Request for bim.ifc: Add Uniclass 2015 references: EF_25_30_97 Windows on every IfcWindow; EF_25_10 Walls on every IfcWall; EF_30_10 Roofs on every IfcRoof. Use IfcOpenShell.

First a look at what the model holds.

```python
import ifcopenshell

model = ifcopenshell.open("bim.ifc")
print(model.schema)
print("classifications:", [c.Name for c in model.by_type("IfcClassification")])
for ifc_class in ("IfcDoor", "IfcRoof", "IfcStair", "IfcWall", "IfcWindow"):
    print(ifc_class, len(model.by_type(ifc_class)))
```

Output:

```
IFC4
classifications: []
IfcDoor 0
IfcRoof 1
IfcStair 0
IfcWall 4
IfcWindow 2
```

```python
import ifcopenshell
import ifcopenshell.api.classification

model = ifcopenshell.open("bim.ifc")

system = ifcopenshell.api.classification.add_classification(model, classification="Uniclass 2015")

codes = {
    "IfcWindow": ("EF_25_30_97", "Windows"),
    "IfcWall": ("EF_25_10", "Walls"),
    "IfcRoof": ("EF_30_10", "Roofs"),
}
for ifc_class, (code, name) in codes.items():
    products = model.by_type(ifc_class)
    ifcopenshell.api.classification.add_reference(
        model, products=products, classification=system, identification=code, name=name
    )
    print(code, len(products))

model.write("bim_updated.ifc")
```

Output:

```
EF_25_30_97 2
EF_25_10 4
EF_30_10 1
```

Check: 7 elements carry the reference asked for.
